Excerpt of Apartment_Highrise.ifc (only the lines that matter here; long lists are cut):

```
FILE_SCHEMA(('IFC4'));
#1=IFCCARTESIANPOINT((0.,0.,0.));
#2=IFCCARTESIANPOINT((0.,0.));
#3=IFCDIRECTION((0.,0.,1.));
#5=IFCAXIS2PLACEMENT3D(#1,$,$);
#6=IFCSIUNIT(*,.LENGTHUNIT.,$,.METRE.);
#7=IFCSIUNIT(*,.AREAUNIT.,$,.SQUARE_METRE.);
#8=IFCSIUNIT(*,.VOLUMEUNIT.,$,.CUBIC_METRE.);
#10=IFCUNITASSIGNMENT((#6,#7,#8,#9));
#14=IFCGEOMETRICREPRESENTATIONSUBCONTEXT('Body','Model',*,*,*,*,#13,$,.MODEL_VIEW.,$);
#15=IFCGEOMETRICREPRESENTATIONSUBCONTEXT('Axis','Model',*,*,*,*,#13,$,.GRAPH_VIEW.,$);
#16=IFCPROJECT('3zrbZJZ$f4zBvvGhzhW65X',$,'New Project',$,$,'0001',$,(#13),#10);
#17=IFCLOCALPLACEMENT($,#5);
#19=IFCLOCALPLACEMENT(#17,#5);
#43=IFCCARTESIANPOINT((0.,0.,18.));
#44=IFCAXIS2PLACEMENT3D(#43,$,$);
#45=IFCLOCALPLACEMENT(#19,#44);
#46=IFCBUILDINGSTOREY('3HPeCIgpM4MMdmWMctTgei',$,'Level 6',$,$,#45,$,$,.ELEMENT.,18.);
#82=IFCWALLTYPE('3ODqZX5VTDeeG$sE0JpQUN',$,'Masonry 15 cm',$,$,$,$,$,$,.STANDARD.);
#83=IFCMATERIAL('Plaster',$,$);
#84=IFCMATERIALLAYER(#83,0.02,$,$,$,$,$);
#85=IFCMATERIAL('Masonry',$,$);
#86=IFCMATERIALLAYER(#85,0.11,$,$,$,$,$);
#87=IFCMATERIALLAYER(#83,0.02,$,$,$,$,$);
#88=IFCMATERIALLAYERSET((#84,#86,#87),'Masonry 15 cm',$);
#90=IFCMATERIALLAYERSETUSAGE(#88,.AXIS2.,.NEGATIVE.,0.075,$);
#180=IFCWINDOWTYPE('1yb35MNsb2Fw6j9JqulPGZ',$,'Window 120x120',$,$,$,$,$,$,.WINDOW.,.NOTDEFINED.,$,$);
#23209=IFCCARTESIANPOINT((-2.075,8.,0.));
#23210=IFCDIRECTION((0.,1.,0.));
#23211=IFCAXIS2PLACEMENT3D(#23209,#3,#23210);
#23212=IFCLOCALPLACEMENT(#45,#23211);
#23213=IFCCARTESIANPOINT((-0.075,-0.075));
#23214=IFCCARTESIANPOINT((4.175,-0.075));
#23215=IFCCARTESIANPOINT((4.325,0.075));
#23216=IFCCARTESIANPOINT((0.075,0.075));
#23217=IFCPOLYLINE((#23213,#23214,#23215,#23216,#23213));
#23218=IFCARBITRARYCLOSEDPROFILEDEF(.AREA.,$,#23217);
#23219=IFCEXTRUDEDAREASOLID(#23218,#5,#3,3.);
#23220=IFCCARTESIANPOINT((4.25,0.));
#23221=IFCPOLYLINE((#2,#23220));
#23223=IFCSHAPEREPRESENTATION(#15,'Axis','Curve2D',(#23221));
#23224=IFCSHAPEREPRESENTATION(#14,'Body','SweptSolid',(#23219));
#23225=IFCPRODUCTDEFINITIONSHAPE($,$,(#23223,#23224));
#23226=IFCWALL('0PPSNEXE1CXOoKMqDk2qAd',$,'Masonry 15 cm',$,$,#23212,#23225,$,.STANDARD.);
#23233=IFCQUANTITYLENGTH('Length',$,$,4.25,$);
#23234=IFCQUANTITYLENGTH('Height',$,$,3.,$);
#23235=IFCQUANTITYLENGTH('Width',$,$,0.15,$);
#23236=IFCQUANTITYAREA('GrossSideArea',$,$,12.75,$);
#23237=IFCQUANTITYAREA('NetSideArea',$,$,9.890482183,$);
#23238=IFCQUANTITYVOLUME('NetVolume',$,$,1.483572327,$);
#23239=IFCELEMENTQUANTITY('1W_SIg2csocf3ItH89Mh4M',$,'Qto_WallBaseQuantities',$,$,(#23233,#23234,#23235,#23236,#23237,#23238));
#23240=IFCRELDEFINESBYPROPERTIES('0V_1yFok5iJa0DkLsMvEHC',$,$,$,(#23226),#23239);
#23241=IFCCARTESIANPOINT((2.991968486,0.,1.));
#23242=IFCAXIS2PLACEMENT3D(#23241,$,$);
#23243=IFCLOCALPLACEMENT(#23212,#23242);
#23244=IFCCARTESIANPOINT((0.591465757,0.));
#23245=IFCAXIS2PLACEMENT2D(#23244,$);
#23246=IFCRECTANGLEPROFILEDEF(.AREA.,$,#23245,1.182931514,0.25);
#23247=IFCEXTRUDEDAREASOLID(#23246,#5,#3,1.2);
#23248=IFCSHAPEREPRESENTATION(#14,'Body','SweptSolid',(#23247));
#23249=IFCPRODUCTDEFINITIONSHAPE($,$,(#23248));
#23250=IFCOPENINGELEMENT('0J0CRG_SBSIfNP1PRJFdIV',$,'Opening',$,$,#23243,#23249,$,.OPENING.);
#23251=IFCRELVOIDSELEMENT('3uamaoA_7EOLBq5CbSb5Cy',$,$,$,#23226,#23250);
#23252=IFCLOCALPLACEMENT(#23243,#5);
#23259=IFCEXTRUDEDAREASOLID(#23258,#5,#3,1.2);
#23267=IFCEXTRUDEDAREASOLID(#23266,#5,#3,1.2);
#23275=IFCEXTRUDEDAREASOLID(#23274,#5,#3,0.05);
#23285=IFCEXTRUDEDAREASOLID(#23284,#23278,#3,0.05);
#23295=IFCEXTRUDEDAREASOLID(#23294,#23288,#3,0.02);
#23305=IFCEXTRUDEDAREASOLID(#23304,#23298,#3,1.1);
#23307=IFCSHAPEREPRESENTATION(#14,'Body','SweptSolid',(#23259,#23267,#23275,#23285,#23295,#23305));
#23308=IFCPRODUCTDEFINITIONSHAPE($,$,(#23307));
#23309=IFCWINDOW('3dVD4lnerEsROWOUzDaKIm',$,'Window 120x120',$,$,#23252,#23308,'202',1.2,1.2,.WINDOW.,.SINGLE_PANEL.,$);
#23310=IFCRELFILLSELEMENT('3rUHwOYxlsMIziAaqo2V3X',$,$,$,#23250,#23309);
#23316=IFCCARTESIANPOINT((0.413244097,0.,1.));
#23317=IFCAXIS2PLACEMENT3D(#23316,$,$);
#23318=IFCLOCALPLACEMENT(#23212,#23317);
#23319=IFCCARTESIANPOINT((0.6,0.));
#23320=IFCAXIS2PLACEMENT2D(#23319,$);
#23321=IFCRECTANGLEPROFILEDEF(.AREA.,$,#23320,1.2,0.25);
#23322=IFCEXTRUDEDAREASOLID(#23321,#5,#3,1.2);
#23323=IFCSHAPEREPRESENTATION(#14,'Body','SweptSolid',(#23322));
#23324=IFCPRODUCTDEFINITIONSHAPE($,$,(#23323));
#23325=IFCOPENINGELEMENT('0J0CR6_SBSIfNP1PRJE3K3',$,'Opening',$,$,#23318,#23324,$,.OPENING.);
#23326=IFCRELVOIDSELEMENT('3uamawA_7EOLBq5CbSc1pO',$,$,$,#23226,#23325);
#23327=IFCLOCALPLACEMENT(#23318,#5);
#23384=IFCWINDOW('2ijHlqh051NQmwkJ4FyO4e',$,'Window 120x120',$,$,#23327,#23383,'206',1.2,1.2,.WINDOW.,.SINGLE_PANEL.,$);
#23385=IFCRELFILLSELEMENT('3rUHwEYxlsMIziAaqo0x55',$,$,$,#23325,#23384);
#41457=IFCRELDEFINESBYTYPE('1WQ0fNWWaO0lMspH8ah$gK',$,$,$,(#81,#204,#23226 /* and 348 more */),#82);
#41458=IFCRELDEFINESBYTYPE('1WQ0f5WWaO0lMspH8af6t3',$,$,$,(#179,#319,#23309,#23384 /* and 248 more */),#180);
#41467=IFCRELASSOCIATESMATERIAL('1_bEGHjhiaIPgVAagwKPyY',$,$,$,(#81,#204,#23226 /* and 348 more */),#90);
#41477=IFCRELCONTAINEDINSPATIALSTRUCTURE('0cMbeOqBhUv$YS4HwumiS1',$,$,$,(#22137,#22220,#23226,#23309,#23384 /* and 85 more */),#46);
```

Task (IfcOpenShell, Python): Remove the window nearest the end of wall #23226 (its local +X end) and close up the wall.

```python
import ifcopenshell
import ifcopenshell.api.feature
import ifcopenshell.api.pset
import ifcopenshell.api.root
import ifcopenshell.geom
import ifcopenshell.util.element
import ifcopenshell.util.shape
import ifcopenshell.util.unit

model = ifcopenshell.open("Apartment_Highrise.ifc")
area_scale = ifcopenshell.util.unit.calculate_unit_scale(model, "AREAUNIT")
volume_scale = ifcopenshell.util.unit.calculate_unit_scale(model, "VOLUMEUNIT")
settings = ifcopenshell.geom.settings()


def volume(element):
    """Net volume in cubic metres, openings subtracted."""
    shape = ifcopenshell.geom.create_shape(settings, element)
    return ifcopenshell.util.shape.get_volume(shape.geometry)


window = model.by_guid("3dVD4lnerEsROWOUzDaKIm")
opening = window.FillsVoids[0].RelatingOpeningElement
wall = opening.VoidsElements[0].RelatingBuildingElement
before = volume(wall)

ifcopenshell.api.root.remove_product(model, product=window)
ifcopenshell.api.feature.remove_feature(model, feature=opening)

after = volume(wall)
thickness = 0.15  # wall thickness in metres

# Update the wall's stored quantities.
qto = model.by_id(ifcopenshell.util.element.get_pset(wall, "Qto_WallBaseQuantities", should_inherit=False)["id"])
ifcopenshell.api.pset.edit_qto(model, qto=qto, properties={
    "NetSideArea": after / thickness / area_scale,
    "NetVolume": after / volume_scale,
})

print(f"wall volume {before:.3f} -> {after:.3f} m3")

model.write("Apartment_Highrise_v2.ifc")
```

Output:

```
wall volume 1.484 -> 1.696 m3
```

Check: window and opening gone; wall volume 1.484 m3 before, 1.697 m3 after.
